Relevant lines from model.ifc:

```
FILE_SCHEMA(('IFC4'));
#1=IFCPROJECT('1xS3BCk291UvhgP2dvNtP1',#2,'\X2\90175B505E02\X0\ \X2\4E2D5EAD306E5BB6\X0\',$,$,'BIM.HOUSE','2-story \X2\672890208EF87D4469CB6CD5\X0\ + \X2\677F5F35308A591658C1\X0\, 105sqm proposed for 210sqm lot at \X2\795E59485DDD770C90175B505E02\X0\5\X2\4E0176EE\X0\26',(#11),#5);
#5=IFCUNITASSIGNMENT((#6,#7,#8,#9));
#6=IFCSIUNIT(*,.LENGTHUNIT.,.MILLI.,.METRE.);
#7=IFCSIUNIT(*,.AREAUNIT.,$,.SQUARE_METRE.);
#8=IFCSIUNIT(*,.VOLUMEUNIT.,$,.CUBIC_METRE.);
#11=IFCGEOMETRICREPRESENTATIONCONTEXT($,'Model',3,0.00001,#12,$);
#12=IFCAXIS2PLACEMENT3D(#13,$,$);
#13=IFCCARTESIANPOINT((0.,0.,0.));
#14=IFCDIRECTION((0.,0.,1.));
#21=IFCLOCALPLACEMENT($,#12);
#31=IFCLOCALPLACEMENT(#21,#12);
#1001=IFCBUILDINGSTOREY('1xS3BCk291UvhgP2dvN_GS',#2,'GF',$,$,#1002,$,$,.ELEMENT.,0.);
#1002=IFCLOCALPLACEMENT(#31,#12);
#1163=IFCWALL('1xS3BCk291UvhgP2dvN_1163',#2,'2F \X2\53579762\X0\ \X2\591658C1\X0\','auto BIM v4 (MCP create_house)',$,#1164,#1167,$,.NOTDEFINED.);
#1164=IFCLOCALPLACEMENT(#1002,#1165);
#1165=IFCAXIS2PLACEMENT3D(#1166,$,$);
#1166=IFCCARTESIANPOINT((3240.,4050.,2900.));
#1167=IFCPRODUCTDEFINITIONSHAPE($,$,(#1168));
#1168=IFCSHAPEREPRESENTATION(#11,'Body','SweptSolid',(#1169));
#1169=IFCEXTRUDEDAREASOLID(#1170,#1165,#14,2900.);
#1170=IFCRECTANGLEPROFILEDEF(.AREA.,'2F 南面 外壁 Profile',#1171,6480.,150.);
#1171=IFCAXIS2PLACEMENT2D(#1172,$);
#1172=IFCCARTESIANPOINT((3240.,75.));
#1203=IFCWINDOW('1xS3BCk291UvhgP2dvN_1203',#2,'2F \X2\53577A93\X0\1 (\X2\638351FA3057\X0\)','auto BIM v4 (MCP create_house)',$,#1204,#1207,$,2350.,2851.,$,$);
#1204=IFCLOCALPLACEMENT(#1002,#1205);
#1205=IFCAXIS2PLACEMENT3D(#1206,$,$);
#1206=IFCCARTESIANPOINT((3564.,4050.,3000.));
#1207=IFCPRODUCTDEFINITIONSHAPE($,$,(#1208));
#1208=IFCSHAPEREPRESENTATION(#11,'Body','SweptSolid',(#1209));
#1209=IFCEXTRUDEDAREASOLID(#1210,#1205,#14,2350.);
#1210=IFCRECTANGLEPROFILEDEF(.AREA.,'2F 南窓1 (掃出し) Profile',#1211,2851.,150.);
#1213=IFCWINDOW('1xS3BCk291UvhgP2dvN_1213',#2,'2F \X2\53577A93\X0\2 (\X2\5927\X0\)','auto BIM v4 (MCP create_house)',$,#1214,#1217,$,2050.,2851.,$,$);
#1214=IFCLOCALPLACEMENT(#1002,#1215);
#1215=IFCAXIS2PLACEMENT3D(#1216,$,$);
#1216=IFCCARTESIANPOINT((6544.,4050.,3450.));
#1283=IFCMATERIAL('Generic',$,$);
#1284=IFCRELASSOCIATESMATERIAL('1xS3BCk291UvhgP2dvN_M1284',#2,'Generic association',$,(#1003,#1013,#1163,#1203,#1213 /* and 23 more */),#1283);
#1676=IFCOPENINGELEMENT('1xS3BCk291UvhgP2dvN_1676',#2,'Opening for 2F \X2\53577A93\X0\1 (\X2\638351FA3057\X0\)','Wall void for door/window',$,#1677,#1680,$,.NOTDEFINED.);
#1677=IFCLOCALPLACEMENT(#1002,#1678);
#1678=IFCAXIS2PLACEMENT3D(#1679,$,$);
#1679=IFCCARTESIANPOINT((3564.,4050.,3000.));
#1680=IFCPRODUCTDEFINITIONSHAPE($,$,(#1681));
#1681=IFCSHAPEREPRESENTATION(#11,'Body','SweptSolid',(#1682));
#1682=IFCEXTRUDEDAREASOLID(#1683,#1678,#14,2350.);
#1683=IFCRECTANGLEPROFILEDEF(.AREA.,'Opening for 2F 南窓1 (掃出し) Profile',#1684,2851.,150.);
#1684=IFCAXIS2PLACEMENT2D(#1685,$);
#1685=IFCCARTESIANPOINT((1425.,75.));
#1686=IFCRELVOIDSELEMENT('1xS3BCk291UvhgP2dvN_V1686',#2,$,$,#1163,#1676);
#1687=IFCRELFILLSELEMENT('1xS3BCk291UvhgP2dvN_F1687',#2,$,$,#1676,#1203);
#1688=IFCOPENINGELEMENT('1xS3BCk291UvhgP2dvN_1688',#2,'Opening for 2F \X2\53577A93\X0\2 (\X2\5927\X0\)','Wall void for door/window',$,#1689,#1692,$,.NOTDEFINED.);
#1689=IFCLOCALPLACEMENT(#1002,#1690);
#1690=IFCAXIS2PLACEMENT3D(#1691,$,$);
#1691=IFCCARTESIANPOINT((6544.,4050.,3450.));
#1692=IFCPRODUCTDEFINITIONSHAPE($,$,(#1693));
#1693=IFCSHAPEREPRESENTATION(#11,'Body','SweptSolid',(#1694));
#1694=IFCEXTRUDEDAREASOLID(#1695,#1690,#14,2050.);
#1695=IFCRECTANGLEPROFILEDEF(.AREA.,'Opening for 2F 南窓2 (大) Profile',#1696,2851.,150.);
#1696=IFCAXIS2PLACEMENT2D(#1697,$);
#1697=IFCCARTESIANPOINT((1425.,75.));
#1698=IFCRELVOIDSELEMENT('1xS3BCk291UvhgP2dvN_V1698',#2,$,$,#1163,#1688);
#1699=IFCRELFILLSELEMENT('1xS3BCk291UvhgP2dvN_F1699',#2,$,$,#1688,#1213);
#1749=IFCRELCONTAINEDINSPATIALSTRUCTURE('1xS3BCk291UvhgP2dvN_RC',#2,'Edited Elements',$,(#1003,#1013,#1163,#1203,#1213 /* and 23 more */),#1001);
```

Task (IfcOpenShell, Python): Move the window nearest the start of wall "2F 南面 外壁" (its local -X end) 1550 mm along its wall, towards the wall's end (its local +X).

```python
import ifcopenshell
import ifcopenshell.api.geometry
import ifcopenshell.util.placement
import ifcopenshell.util.unit

model = ifcopenshell.open("model.ifc")
unit_scale = ifcopenshell.util.unit.calculate_unit_scale(model)

window = model.by_guid("1xS3BCk291UvhgP2dvN_1203")
opening = window.FillsVoids[0].RelatingOpeningElement
wall = opening.VoidsElements[0].RelatingBuildingElement

wall_matrix = ifcopenshell.util.placement.get_local_placement(wall.ObjectPlacement)
shift = wall_matrix[:3, 0] * 1.55 / unit_scale
before = ifcopenshell.util.placement.get_local_placement(window.ObjectPlacement)[:3, 3].copy()

# The window is not placed relative to its opening, so move both.
for product in (opening, window):
    matrix = ifcopenshell.util.placement.get_local_placement(product.ObjectPlacement)
    matrix[:3, 3] += shift
    ifcopenshell.api.geometry.edit_object_placement(model, product=product, matrix=matrix, is_si=False)

after = ifcopenshell.util.placement.get_local_placement(window.ObjectPlacement)[:3, 3]
print("window moved by", (after - before).round(3) + 0.0)

model.write("model_updated.ifc")
```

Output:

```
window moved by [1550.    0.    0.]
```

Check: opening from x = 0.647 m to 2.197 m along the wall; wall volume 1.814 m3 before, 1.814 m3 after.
